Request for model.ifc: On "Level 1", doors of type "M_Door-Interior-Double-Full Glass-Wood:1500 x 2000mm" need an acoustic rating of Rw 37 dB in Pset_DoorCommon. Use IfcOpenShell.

First a look at what the model holds.

```python
import ifcopenshell
import ifcopenshell.util.element

model = ifcopenshell.open("model.ifc")
print(model.schema)
storey = next(s for s in model.by_type("IfcBuildingStorey") if s.Name == "Level 1")
doors = [e for e in ifcopenshell.util.element.get_decomposition(storey) if e.is_a("IfcDoor")]
seen = {}
for e in doors:
    element_type = ifcopenshell.util.element.get_type(e)
    key = (element_type.Name if element_type != e and element_type else None, ifcopenshell.util.element.get_pset(e, "Pset_DoorCommon", "AcousticRating"))
    seen[key] = seen.get(key, 0) + 1
for (name, value), count in sorted(seen.items(), key=str):
    print(count, "x", name, "|", value)
```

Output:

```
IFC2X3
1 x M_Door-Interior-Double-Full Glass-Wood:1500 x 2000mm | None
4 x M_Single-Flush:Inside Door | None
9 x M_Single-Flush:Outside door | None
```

```python
import ifcopenshell
import ifcopenshell.api.pset
import ifcopenshell.util.element

model = ifcopenshell.open("model.ifc")

storey = next(s for s in model.by_type("IfcBuildingStorey") if s.Name == "Level 1")
doors = [e for e in ifcopenshell.util.element.get_decomposition(storey) if e.is_a("IfcDoor")]

count = 0
for e in doors:
    element_type = ifcopenshell.util.element.get_type(e)
    if element_type in (None, e) or element_type.Name != "M_Door-Interior-Double-Full Glass-Wood:1500 x 2000mm":
        continue
    # add_pset returns the element's existing set when there is one.
    pset = ifcopenshell.api.pset.add_pset(model, product=e, name="Pset_DoorCommon")
    ifcopenshell.api.pset.edit_pset(model, pset=pset, properties={"AcousticRating": "Rw 37 dB"})
    count += 1

print(count, "doors updated")

model.write("model_rev.ifc")
```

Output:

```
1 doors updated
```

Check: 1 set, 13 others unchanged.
